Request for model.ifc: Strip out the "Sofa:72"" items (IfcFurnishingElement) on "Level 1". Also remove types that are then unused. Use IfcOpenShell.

First a look at what the model holds.

```python
import ifcopenshell
import ifcopenshell.util.element

model = ifcopenshell.open("model.ifc")
print(model.schema)
storey = next(s for s in model.by_type("IfcBuildingStorey") if s.Name == "Level 1")
furniture = [e for e in ifcopenshell.util.element.get_decomposition(storey) if e.is_a("IfcFurnishingElement")]
seen = {}
for e in furniture:
    element_type = ifcopenshell.util.element.get_type(e)
    name = element_type.Name if element_type not in (None, e) else None
    seen[name] = seen.get(name, 0) + 1
for name, count in sorted(seen.items(), key=str):
    print(count, "x", name)
```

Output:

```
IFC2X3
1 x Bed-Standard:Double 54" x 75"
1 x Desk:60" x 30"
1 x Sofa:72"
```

```python
import ifcopenshell
import ifcopenshell.api.root
import ifcopenshell.util.element

model = ifcopenshell.open("model.ifc")

storey = next(s for s in model.by_type("IfcBuildingStorey") if s.Name == "Level 1")
furniture = [e for e in ifcopenshell.util.element.get_decomposition(storey) if e.is_a("IfcFurnishingElement")]
targets = [e for e in furniture if (t := ifcopenshell.util.element.get_type(e)) not in (None, e) and t.Name == 'Sofa:72"']
types = {ifcopenshell.util.element.get_type(e) for e in targets} - {None, *targets}

for e in targets:
    ifcopenshell.api.root.remove_product(model, product=e)
print(len(targets), "removed")

unused = [t for t in types if not ifcopenshell.util.element.get_types(t)]
for t in unused:
    ifcopenshell.api.root.remove_product(model, product=t)
print(len(unused), "unused types removed")

model.write("model_v2.ifc")
```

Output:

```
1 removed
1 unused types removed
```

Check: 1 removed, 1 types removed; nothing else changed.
